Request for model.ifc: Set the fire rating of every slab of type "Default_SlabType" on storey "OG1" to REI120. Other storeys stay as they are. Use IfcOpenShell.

First a look at what the model holds.

```python
import ifcopenshell
import ifcopenshell.util.element

model = ifcopenshell.open("model.ifc")
print(model.schema)
storey = next(s for s in model.by_type("IfcBuildingStorey") if s.Name == "OG1")
slabs = [e for e in ifcopenshell.util.element.get_decomposition(storey) if e.is_a("IfcSlab")]
seen = {}
for e in slabs:
    element_type = ifcopenshell.util.element.get_type(e)
    key = (element_type.Name if element_type != e and element_type else None, ifcopenshell.util.element.get_pset(e, "Pset_SlabCommon", "FireRating"))
    seen[key] = seen.get(key, 0) + 1
for (name, value), count in sorted(seen.items(), key=str):
    print(count, "x", name, "|", value)
```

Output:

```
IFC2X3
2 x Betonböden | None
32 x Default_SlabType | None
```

```python
import ifcopenshell
import ifcopenshell.api.pset
import ifcopenshell.util.element

model = ifcopenshell.open("model.ifc")

storey = next(s for s in model.by_type("IfcBuildingStorey") if s.Name == "OG1")
slabs = [e for e in ifcopenshell.util.element.get_decomposition(storey) if e.is_a("IfcSlab")]

count = 0
for e in slabs:
    element_type = ifcopenshell.util.element.get_type(e)
    if element_type in (None, e) or element_type.Name != "Default_SlabType":
        continue
    # add_pset returns the element's existing set when there is one.
    pset = ifcopenshell.api.pset.add_pset(model, product=e, name="Pset_SlabCommon")
    ifcopenshell.api.pset.edit_pset(model, pset=pset, properties={"FireRating": "REI120"})
    count += 1

print(count, "slabs updated")

model.write("model-out.ifc")
```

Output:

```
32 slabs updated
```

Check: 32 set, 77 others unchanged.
